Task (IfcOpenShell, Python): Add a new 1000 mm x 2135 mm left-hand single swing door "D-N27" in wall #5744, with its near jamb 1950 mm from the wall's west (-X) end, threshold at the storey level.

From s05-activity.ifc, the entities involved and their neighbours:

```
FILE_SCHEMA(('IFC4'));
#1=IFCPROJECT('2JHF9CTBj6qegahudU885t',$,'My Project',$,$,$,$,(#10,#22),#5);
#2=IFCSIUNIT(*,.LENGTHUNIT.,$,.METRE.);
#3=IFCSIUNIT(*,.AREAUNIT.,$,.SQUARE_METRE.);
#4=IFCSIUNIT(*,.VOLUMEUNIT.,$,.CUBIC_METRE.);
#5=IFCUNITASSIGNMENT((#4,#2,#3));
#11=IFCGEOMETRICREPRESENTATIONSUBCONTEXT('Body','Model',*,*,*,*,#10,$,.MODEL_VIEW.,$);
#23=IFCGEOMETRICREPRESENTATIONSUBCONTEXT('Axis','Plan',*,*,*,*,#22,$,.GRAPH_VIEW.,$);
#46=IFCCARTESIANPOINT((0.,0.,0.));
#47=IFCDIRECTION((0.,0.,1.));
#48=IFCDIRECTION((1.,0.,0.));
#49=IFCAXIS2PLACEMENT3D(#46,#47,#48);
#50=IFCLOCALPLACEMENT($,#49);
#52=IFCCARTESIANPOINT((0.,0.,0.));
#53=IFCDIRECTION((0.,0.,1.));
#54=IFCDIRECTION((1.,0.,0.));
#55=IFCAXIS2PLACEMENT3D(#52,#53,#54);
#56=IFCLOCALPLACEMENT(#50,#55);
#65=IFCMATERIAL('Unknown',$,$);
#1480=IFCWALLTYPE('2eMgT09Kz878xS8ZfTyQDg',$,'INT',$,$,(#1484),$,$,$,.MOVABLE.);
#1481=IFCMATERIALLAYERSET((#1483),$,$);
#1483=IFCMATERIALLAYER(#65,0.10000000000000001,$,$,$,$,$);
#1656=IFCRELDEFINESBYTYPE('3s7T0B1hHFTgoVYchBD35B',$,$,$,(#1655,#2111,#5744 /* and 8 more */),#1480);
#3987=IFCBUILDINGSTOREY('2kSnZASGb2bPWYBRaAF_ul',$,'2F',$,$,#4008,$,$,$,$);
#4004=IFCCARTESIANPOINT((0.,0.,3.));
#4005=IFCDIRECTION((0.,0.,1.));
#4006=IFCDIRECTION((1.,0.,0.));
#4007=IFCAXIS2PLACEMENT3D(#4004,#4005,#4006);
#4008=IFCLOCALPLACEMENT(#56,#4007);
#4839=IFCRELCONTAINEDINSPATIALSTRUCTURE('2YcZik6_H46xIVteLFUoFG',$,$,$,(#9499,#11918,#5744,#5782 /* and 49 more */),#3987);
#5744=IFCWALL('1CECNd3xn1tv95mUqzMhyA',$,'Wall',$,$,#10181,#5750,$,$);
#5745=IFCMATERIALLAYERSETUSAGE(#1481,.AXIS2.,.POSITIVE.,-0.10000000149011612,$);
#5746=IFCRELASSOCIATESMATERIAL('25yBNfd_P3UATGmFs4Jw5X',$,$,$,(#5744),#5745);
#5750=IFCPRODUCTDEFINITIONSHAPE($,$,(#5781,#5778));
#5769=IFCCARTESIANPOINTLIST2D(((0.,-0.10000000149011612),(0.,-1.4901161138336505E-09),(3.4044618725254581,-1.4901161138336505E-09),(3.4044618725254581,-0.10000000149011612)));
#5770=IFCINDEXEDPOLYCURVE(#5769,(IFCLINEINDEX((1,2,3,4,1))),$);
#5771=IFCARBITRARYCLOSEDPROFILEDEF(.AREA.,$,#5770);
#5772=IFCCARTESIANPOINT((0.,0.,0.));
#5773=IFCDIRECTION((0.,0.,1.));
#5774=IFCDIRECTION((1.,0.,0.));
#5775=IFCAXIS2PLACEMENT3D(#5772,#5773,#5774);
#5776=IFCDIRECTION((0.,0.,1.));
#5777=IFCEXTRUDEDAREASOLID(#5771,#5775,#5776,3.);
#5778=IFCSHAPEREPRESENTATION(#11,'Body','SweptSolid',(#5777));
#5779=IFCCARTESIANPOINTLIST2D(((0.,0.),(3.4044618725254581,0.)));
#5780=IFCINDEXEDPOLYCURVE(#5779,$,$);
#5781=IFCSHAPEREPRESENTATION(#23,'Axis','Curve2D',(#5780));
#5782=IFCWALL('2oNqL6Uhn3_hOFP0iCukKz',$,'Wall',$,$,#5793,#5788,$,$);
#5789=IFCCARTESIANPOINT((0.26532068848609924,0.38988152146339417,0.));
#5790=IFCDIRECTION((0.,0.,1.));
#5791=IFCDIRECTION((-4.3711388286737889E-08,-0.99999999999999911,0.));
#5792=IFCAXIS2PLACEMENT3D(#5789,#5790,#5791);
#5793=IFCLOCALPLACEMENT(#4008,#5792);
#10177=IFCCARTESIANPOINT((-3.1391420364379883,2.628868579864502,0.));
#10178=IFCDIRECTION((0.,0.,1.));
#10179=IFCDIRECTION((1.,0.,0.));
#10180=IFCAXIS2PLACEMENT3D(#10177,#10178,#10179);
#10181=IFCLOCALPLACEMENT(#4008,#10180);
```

```python
import numpy as np
import ifcopenshell
import ifcopenshell.api.feature
import ifcopenshell.api.geometry
import ifcopenshell.api.root
import ifcopenshell.api.spatial
import ifcopenshell.geom
import ifcopenshell.util.element
import ifcopenshell.util.placement
import ifcopenshell.util.representation
import ifcopenshell.util.shape
import ifcopenshell.util.unit

model = ifcopenshell.open("s05-activity.ifc")
unit_scale = ifcopenshell.util.unit.calculate_unit_scale(model)
settings = ifcopenshell.geom.settings()


def volume(element):
    """Net volume in cubic metres, openings subtracted."""
    shape = ifcopenshell.geom.create_shape(settings, element)
    return ifcopenshell.util.shape.get_volume(shape.geometry)


wall = model.by_guid("1CECNd3xn1tv95mUqzMhyA")
storey = ifcopenshell.util.element.get_container(wall, ifc_class="IfcBuildingStorey")
context = ifcopenshell.util.representation.get_context(model, "Model", "Body", "MODEL_VIEW")
before = volume(wall)

width, height, from_end, sill = 1, 2.135, 1.95, 0.0  # metres

# The wall runs along its own X axis, and the end named is its -X end.
wall_shape = ifcopenshell.geom.create_shape(settings, wall)
x, y, z = ifcopenshell.util.shape.get_vertices(wall_shape.geometry).T
start = x.min() + from_end
face, thickness = float(y.min()), float(y.max() - y.min())
wall_matrix = ifcopenshell.util.placement.get_local_placement(wall.ObjectPlacement)
level = ifcopenshell.util.placement.get_local_placement(storey.ObjectPlacement)[2, 3]


def in_wall(x, y):
    """Placement at x, y metres in the wall's axes, at sill height."""
    matrix = wall_matrix.copy()
    matrix[:, 3] = wall_matrix @ np.array([x / unit_scale, y / unit_scale, 0.0, 1.0])
    matrix[2, 3] = level + sill / unit_scale
    return matrix


# Opening: a box that overshoots both wall faces by 50 mm.
opening = ifcopenshell.api.root.create_entity(model, ifc_class="IfcOpeningElement", predefined_type="OPENING")
box = ifcopenshell.api.geometry.add_wall_representation(
    model, context=context, length=width, height=height, thickness=thickness + 0.1
)
ifcopenshell.api.geometry.assign_representation(model, product=opening, representation=box)
ifcopenshell.api.geometry.edit_object_placement(model, product=opening, matrix=in_wall(start, face - 0.05), is_si=False)
ifcopenshell.api.feature.add_feature(model, feature=opening, element=wall)

door = ifcopenshell.api.root.create_entity(model, ifc_class="IfcDoor", name="D-N27", predefined_type="DOOR")
door.OverallWidth, door.OverallHeight = width / unit_scale, height / unit_scale
door.OperationType = "SINGLE_SWING_LEFT"
body = ifcopenshell.api.geometry.add_door_representation(
    model,
    context=context,
    overall_width=door.OverallWidth,
    overall_height=door.OverallHeight,
    operation_type="SINGLE_SWING_LEFT",
    lining_properties={"LiningDepth": thickness / unit_scale, "ThresholdDepth": thickness / unit_scale},
)
ifcopenshell.api.geometry.assign_representation(model, product=door, representation=body)
ifcopenshell.api.spatial.assign_container(model, products=[door], relating_structure=storey)
ifcopenshell.api.feature.add_filling(model, opening=opening, element=door)

# The lining spans the wall, so the door starts at the wall face.
ifcopenshell.api.geometry.edit_object_placement(model, product=door, matrix=in_wall(start, face), is_si=False)

after = volume(wall)

print(f"wall volume {before:.3f} -> {after:.3f} m3")

model.write("s05-activity_rev.ifc")
```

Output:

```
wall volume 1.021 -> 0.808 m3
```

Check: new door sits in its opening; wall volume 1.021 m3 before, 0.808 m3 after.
